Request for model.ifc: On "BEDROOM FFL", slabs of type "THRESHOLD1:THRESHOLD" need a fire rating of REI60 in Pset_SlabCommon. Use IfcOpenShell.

First a look at what the model holds.

```python
import ifcopenshell
import ifcopenshell.util.element

model = ifcopenshell.open("model.ifc")
print(model.schema)
storey = next(s for s in model.by_type("IfcBuildingStorey") if s.Name == "BEDROOM FFL")
slabs = [e for e in ifcopenshell.util.element.get_decomposition(storey) if e.is_a("IfcSlab")]
seen = {}
for e in slabs:
    element_type = ifcopenshell.util.element.get_type(e)
    key = (element_type.Name if element_type != e and element_type else None, ifcopenshell.util.element.get_pset(e, "Pset_SlabCommon", "FireRating"))
    seen[key] = seen.get(key, 0) + 1
for (name, value), count in sorted(seen.items(), key=str):
    print(count, "x", name, "|", value)
```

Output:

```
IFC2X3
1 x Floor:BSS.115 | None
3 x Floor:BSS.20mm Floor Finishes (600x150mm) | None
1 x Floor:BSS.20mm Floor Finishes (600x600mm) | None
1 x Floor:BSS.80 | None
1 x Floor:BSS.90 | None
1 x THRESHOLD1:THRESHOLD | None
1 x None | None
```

```python
import ifcopenshell
import ifcopenshell.api.pset
import ifcopenshell.util.element

model = ifcopenshell.open("model.ifc")

storey = next(s for s in model.by_type("IfcBuildingStorey") if s.Name == "BEDROOM FFL")
slabs = [e for e in ifcopenshell.util.element.get_decomposition(storey) if e.is_a("IfcSlab")]

count = 0
for e in slabs:
    element_type = ifcopenshell.util.element.get_type(e)
    if element_type in (None, e) or element_type.Name != "THRESHOLD1:THRESHOLD":
        continue
    # add_pset returns the element's existing set when there is one.
    pset = ifcopenshell.api.pset.add_pset(model, product=e, name="Pset_SlabCommon")
    ifcopenshell.api.pset.edit_pset(model, pset=pset, properties={"FireRating": "REI60"})
    count += 1

print(count, "slabs updated")

model.write("model_edited.ifc")
```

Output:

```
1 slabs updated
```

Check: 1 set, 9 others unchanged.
